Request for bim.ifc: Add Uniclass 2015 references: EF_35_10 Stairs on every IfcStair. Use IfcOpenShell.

First a look at what the model holds.

```python
import ifcopenshell

model = ifcopenshell.open("bim.ifc")
print(model.schema)
print("classifications:", [c.Name for c in model.by_type("IfcClassification")])
for ifc_class in ("IfcDoor", "IfcRoof", "IfcStair", "IfcWall", "IfcWindow"):
    print(ifc_class, len(model.by_type(ifc_class)))
```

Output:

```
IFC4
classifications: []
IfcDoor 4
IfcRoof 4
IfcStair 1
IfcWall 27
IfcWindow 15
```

```python
import ifcopenshell
import ifcopenshell.api.classification

model = ifcopenshell.open("bim.ifc")

system = ifcopenshell.api.classification.add_classification(model, classification="Uniclass 2015")

codes = {
    "IfcStair": ("EF_35_10", "Stairs"),
}
for ifc_class, (code, name) in codes.items():
    products = model.by_type(ifc_class)
    ifcopenshell.api.classification.add_reference(
        model, products=products, classification=system, identification=code, name=name
    )
    print(code, len(products))

model.write("bim_updated.ifc")
```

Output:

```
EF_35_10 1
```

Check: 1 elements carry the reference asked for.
